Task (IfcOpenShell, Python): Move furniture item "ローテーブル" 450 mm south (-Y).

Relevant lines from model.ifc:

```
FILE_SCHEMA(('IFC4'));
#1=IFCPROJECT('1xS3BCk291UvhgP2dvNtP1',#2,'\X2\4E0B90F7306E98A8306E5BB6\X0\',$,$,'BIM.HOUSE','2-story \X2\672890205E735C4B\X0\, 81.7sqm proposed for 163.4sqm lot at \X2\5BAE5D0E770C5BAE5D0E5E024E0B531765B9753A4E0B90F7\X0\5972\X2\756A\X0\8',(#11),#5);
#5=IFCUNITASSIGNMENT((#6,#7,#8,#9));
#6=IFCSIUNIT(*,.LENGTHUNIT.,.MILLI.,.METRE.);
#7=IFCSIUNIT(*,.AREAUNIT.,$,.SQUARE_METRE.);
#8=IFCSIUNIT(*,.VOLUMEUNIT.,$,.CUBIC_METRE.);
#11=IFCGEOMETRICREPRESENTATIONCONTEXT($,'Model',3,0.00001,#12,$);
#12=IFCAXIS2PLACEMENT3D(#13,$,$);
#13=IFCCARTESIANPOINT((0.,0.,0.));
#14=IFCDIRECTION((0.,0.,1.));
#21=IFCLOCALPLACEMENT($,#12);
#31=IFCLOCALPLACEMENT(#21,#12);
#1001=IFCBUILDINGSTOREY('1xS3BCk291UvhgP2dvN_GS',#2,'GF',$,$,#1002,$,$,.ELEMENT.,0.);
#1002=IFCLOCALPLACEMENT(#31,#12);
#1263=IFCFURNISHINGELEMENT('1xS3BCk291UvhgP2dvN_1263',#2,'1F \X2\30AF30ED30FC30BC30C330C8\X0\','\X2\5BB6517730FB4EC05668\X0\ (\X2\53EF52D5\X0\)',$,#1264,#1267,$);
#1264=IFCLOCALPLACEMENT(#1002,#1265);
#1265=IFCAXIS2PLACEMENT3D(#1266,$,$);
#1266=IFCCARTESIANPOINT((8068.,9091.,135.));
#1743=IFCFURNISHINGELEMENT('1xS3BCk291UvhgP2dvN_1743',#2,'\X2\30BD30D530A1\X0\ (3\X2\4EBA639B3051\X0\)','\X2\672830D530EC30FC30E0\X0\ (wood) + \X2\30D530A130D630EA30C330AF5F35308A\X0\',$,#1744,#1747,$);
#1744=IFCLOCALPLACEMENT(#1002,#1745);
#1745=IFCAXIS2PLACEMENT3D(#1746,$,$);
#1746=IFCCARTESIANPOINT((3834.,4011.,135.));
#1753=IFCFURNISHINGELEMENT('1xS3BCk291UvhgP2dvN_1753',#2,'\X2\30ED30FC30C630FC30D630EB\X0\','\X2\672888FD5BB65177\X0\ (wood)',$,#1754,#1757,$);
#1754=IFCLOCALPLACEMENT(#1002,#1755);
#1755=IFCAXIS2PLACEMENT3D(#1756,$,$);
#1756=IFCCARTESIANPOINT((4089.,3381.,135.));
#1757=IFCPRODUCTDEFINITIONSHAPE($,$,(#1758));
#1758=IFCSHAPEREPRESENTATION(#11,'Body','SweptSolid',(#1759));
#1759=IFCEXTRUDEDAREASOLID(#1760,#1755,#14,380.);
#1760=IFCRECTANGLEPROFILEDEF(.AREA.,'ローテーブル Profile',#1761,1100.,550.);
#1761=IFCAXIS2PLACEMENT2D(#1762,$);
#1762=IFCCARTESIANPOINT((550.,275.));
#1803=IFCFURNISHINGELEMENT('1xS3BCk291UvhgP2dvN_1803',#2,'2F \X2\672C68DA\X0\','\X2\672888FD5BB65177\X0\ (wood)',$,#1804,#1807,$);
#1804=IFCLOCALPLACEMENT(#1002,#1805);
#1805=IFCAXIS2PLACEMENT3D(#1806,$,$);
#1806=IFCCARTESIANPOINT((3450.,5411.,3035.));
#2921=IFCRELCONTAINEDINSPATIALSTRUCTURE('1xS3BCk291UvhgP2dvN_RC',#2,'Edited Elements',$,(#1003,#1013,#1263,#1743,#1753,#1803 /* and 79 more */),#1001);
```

```python
import ifcopenshell
import ifcopenshell.api.geometry
import ifcopenshell.util.placement
import ifcopenshell.util.unit

model = ifcopenshell.open("model.ifc")
unit_scale = ifcopenshell.util.unit.calculate_unit_scale(model)

item = model.by_guid("1xS3BCk291UvhgP2dvN_1753")
matrix = ifcopenshell.util.placement.get_local_placement(item.ObjectPlacement)
matrix[1, 3] -= 0.45 / unit_scale
ifcopenshell.api.geometry.edit_object_placement(model, product=item, matrix=matrix, is_si=False)

print(ifcopenshell.util.placement.get_local_placement(item.ObjectPlacement).round(3) + 0.0)

model.write("model-out.ifc")
```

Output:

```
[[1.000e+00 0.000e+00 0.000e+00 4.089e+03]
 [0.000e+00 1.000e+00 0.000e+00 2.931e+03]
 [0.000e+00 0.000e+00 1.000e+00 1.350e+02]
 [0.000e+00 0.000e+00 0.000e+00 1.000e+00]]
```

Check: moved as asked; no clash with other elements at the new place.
